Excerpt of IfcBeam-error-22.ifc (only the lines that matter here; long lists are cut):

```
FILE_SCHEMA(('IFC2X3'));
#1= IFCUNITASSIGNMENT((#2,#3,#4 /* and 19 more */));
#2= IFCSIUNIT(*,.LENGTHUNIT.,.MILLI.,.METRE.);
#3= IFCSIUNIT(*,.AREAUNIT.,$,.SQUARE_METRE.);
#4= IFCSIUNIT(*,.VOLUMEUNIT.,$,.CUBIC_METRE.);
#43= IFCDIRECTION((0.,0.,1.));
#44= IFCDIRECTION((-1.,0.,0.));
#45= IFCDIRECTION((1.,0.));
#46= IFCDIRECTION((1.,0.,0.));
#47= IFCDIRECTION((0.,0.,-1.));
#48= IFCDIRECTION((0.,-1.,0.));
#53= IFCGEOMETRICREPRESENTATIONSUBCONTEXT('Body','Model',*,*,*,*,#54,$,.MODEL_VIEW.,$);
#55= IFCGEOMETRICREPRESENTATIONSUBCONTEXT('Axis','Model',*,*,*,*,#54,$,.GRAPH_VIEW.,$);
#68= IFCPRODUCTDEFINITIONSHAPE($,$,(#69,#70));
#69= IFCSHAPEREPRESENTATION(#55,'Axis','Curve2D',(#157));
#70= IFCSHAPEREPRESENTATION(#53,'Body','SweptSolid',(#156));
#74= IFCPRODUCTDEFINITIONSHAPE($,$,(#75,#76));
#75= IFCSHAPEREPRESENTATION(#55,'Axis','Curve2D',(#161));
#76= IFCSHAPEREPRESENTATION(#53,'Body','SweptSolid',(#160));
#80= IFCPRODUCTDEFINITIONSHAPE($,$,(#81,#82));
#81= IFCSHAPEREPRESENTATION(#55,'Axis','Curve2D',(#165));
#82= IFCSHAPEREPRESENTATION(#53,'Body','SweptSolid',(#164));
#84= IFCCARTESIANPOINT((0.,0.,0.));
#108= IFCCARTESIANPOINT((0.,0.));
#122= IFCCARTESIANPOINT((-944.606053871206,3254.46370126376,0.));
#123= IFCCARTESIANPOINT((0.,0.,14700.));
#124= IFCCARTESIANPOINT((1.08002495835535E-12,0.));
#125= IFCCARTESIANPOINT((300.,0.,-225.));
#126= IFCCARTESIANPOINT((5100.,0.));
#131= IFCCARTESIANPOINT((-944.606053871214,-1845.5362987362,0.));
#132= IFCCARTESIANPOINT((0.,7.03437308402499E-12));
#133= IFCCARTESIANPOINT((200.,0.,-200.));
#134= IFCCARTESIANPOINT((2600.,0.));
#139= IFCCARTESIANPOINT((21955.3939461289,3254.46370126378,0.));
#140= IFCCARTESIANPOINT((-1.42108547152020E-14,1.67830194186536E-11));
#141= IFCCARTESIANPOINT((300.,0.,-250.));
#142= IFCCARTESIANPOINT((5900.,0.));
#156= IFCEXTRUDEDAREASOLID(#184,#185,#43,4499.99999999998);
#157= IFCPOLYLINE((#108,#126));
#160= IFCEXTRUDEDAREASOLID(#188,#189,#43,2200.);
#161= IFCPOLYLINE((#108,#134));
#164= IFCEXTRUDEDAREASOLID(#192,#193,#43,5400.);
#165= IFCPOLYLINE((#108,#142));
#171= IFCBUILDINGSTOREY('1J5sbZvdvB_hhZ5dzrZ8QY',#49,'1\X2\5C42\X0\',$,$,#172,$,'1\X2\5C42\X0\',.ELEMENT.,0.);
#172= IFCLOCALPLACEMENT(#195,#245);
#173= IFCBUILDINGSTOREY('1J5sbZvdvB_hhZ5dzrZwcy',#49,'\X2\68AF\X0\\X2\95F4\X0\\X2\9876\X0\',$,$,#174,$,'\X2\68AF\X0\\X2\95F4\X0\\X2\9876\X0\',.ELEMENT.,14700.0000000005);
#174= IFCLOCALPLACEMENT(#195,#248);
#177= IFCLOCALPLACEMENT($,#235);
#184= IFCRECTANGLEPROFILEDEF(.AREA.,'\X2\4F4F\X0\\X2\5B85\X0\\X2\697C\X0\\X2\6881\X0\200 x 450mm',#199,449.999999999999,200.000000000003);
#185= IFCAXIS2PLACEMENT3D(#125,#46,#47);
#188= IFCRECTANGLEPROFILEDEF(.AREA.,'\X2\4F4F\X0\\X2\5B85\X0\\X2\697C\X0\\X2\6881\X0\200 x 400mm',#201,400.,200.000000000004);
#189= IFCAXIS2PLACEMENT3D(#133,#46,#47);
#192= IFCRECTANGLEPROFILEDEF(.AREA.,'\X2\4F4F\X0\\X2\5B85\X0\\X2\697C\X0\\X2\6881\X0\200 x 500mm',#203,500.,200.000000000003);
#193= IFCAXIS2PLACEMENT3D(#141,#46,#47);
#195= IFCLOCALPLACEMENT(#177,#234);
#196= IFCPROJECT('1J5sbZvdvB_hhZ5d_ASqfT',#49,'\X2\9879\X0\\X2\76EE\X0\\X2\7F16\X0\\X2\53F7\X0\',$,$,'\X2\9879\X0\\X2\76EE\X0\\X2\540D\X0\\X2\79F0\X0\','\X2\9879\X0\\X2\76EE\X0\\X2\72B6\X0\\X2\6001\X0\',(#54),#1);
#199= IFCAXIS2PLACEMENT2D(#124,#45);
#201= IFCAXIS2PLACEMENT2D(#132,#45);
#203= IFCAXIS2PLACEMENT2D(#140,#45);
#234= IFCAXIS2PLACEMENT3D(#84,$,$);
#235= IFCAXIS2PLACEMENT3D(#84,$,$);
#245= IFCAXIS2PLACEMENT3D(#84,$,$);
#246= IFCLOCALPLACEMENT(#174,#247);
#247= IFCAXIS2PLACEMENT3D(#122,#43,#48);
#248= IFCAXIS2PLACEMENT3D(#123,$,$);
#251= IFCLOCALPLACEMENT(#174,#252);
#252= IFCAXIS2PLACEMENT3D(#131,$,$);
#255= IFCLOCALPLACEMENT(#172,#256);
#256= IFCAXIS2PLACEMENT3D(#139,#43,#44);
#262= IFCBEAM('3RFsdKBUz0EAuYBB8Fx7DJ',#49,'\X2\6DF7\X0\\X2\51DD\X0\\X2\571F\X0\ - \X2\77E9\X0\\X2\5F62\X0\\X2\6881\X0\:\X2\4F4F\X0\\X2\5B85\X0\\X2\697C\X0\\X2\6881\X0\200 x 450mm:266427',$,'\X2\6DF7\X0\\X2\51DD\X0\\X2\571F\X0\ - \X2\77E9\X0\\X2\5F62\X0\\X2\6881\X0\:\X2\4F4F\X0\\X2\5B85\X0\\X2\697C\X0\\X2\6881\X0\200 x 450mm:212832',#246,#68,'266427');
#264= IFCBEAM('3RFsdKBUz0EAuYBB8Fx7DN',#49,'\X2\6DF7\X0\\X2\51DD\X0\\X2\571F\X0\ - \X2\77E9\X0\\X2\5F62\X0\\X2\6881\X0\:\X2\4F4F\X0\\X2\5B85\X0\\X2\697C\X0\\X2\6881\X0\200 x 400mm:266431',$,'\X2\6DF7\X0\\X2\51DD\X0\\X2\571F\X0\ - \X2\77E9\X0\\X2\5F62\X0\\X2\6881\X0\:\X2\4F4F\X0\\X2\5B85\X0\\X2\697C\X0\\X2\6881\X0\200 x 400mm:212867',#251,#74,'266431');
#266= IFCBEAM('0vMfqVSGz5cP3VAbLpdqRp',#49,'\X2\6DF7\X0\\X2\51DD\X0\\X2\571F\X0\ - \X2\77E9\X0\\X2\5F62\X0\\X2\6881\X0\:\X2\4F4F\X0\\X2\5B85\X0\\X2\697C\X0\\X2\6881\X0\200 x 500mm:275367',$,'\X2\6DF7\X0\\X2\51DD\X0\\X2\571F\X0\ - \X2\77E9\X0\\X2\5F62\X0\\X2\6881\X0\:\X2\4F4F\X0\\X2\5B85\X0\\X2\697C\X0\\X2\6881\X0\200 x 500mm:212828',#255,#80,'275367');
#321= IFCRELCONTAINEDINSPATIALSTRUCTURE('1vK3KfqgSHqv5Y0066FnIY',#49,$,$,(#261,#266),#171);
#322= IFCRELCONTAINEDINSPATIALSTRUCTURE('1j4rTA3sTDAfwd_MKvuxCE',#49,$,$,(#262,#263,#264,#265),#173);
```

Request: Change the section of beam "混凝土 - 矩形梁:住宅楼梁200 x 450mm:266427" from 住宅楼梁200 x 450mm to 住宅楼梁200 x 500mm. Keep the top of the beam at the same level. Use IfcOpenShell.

```python
import ifcopenshell
import ifcopenshell.util.element
import ifcopenshell.util.representation

model = ifcopenshell.open("IfcBeam-error-22.ifc")

member = model.by_id(262)
source = next(p for p in model.by_type("IfcRectangleProfileDef") if p.ProfileName == "住宅楼梁200 x 500mm")

body = ifcopenshell.util.representation.get_representation(member, "Model", "Body")
solid = body.Items[0]
old_profile = solid.SweptArea

# Copy the section's sizes but keep this member's own profile position.
profile = ifcopenshell.util.element.copy(model, source)
# Profiles are centred, so shift by half the change in depth to hold the top.
shift = (old_profile.XDim - profile.XDim) / 2
x, y = old_profile.Position.Location.Coordinates
up = (-1.0, 0.0)  # upwards, in the solid's own plane
location = model.createIfcCartesianPoint((x + up[0] * shift, y + up[1] * shift))
profile.Position = model.createIfcAxis2Placement2D(location, old_profile.Position.RefDirection)
solid.SweptArea = profile
if not model.get_total_inverses(old_profile):
    ifcopenshell.util.element.remove_deep2(model, old_profile)
member.Name = member.Name.replace("住宅楼梁200 x 450mm", "住宅楼梁200 x 500mm")
member.ObjectType = member.ObjectType.replace("住宅楼梁200 x 450mm", "住宅楼梁200 x 500mm")

print(solid.SweptArea)

model.write("IfcBeam-error-22_edited.ifc")
```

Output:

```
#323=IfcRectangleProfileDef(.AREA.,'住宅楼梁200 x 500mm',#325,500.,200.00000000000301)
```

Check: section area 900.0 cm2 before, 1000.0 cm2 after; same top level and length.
